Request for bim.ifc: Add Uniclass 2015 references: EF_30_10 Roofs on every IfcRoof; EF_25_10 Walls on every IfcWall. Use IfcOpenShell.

First a look at what the model holds.

```python
import ifcopenshell

model = ifcopenshell.open("bim.ifc")
print(model.schema)
print("classifications:", [c.Name for c in model.by_type("IfcClassification")])
for ifc_class in ("IfcDoor", "IfcRoof", "IfcStair", "IfcWall", "IfcWindow"):
    print(ifc_class, len(model.by_type(ifc_class)))
```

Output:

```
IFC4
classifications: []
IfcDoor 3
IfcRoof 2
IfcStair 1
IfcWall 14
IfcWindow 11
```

```python
import ifcopenshell
import ifcopenshell.api.classification

model = ifcopenshell.open("bim.ifc")

system = ifcopenshell.api.classification.add_classification(model, classification="Uniclass 2015")

codes = {
    "IfcRoof": ("EF_30_10", "Roofs"),
    "IfcWall": ("EF_25_10", "Walls"),
}
for ifc_class, (code, name) in codes.items():
    products = model.by_type(ifc_class)
    ifcopenshell.api.classification.add_reference(
        model, products=products, classification=system, identification=code, name=name
    )
    print(code, len(products))

model.write("bim_v2.ifc")
```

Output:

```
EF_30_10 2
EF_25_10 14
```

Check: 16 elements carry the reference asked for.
